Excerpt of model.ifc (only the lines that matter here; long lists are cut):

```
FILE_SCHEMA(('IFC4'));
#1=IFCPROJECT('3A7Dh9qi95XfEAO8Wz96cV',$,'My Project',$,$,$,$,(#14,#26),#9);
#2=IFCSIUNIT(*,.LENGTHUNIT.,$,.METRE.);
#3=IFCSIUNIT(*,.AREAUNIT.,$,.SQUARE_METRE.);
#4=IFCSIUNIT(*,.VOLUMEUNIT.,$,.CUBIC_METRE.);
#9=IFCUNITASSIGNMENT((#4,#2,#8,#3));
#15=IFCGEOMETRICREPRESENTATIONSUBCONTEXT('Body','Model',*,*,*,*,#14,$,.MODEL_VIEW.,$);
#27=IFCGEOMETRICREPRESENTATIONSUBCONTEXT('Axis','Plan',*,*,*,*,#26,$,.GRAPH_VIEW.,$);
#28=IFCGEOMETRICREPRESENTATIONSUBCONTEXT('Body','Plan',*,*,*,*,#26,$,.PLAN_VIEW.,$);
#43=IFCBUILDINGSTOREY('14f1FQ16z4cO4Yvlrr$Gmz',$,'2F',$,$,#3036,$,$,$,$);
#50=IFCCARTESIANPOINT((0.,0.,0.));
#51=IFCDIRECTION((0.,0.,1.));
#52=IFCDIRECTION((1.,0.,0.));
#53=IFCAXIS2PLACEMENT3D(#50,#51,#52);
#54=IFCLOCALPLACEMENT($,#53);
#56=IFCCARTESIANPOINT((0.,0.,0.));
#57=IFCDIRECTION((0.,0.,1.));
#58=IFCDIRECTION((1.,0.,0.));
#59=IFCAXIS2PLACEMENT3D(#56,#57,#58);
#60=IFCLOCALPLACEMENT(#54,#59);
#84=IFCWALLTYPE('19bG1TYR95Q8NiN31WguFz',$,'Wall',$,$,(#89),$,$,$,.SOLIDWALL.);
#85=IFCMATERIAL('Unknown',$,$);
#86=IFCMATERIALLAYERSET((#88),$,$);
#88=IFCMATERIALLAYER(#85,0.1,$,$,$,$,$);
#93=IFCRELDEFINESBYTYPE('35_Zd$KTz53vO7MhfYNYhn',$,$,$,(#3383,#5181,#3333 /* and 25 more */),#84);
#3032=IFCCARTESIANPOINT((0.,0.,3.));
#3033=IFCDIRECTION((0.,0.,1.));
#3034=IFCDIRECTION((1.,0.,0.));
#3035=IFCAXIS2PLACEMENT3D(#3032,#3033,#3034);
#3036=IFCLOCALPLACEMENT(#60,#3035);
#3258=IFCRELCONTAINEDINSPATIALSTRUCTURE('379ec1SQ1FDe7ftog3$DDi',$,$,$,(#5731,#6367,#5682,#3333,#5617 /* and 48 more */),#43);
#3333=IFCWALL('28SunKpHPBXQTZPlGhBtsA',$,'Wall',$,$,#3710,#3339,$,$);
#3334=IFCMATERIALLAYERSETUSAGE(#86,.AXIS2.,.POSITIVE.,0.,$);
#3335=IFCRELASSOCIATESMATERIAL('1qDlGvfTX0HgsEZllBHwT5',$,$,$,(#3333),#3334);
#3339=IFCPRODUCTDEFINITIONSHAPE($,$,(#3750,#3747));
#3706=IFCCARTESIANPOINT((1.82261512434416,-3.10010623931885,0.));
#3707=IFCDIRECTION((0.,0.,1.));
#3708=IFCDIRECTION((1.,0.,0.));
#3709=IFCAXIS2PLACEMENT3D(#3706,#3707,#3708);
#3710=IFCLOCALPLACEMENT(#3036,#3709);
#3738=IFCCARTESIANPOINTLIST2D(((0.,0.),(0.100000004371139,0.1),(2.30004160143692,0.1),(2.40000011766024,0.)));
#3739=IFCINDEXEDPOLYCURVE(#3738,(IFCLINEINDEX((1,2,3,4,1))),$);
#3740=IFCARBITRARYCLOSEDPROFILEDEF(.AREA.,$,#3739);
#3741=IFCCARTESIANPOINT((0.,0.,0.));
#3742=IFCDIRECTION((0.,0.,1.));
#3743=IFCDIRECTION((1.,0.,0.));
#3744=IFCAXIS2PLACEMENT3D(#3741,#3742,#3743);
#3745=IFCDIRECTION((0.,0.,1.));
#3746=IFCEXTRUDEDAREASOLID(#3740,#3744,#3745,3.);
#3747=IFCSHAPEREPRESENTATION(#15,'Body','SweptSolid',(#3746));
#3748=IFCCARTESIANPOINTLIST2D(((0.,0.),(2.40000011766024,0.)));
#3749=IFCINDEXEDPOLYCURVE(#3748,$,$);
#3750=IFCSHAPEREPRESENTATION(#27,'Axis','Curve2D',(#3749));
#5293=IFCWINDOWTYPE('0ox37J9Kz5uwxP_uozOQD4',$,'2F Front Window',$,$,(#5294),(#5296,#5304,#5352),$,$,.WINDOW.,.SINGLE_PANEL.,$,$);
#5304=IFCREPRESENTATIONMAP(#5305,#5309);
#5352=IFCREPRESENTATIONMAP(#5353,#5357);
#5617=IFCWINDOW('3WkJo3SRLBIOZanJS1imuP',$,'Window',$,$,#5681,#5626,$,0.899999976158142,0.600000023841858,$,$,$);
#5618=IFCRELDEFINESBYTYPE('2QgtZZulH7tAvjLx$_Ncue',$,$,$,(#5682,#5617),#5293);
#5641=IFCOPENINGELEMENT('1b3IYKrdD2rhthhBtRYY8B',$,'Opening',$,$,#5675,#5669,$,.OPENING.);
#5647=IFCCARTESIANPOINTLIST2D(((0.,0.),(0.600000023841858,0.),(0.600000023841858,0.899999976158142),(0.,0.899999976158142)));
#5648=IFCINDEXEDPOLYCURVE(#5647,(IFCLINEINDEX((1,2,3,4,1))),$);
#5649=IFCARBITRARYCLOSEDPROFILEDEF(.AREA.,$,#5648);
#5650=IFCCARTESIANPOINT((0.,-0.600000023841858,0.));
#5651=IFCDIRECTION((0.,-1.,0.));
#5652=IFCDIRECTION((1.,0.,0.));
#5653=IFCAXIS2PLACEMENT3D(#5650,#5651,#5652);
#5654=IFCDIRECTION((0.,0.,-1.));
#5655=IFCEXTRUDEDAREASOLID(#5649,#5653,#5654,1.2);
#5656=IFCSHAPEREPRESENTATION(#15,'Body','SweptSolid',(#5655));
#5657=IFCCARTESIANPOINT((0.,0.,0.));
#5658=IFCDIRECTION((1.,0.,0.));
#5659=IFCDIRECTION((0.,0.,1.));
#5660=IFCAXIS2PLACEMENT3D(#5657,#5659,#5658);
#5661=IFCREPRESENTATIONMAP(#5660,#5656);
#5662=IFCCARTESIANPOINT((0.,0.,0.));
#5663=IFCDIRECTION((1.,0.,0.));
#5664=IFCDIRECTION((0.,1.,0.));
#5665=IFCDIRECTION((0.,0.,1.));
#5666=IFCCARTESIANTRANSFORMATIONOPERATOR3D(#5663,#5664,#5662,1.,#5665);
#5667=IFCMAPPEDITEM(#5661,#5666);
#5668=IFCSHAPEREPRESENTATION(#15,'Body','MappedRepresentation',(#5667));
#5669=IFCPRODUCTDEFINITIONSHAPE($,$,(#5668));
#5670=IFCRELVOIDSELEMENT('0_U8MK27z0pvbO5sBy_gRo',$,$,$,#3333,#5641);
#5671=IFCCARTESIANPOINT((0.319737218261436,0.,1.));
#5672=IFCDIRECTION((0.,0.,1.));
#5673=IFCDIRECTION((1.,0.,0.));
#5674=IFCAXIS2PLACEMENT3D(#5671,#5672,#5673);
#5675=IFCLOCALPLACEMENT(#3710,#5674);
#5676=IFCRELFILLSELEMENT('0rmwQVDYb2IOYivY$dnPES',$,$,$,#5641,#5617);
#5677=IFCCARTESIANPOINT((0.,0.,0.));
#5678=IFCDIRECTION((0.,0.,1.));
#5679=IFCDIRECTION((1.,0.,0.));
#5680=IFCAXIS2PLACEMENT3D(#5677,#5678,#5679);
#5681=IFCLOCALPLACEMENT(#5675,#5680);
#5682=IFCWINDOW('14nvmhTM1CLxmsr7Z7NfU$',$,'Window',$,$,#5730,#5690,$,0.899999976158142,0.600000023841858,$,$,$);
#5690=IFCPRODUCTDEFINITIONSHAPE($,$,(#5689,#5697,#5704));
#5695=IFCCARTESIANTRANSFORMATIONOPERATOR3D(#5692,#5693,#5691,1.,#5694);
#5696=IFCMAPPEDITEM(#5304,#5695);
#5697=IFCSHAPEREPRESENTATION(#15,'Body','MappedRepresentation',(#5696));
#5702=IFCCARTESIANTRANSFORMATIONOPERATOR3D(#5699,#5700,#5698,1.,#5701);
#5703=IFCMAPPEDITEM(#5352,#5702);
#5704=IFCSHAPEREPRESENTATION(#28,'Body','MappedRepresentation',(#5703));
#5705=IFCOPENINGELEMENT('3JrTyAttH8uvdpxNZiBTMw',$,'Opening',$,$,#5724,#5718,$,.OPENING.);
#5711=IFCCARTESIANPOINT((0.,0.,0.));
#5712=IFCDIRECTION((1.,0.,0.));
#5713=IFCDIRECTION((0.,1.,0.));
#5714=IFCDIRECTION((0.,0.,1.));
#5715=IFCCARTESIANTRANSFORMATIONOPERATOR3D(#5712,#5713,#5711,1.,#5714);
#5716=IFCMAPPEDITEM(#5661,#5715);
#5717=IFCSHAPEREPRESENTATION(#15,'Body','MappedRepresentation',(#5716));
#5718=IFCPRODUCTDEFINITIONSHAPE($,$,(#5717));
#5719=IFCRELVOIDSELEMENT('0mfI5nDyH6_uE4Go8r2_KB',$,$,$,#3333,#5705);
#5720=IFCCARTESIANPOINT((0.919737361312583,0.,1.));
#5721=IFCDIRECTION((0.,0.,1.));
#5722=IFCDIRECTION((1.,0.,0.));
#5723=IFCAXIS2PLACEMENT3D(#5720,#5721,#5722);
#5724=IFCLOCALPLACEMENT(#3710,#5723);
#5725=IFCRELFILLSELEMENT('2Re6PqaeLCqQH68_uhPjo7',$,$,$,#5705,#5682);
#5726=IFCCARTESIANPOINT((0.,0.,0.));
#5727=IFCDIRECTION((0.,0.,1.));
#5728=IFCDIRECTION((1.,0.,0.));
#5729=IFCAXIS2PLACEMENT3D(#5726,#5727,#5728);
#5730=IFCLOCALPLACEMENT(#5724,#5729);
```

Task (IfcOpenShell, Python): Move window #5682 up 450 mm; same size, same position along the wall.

```python
import numpy as np
import ifcopenshell
import ifcopenshell.api.geometry
import ifcopenshell.util.placement
import ifcopenshell.util.unit

model = ifcopenshell.open("model.ifc")
unit_scale = ifcopenshell.util.unit.calculate_unit_scale(model)

window = model.by_guid("14nvmhTM1CLxmsr7Z7NfU$")
opening = window.FillsVoids[0].RelatingOpeningElement
dz = 0.45

shift = np.array([0.0, 0.0, dz])
# The window is placed relative to its opening, so it follows when the opening moves.
matrix = ifcopenshell.util.placement.get_local_placement(opening.ObjectPlacement)
matrix[:3, 3] += shift
ifcopenshell.api.geometry.edit_object_placement(
    model, product=opening, matrix=matrix, is_si=False, should_transform_children=True
)

print(f"moved by {dz * unit_scale:+.3f} m")

model.write("model_v2.ifc")
```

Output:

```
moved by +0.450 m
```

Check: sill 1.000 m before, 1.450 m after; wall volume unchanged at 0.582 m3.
